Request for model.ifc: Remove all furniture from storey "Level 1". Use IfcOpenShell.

First a look at what the model holds.

```python
import ifcopenshell
import ifcopenshell.util.element

model = ifcopenshell.open("model.ifc")
print(model.schema)
storey = next(s for s in model.by_type("IfcBuildingStorey") if s.Name == "Level 1")
furniture = [e for e in ifcopenshell.util.element.get_decomposition(storey) if e.is_a("IfcFurnishingElement")]
seen = {}
for e in furniture:
    element_type = ifcopenshell.util.element.get_type(e)
    name = element_type.Name if element_type not in (None, e) else None
    seen[name] = seen.get(name, 0) + 1
for name, count in sorted(seen.items(), key=str):
    print(count, "x", name)
```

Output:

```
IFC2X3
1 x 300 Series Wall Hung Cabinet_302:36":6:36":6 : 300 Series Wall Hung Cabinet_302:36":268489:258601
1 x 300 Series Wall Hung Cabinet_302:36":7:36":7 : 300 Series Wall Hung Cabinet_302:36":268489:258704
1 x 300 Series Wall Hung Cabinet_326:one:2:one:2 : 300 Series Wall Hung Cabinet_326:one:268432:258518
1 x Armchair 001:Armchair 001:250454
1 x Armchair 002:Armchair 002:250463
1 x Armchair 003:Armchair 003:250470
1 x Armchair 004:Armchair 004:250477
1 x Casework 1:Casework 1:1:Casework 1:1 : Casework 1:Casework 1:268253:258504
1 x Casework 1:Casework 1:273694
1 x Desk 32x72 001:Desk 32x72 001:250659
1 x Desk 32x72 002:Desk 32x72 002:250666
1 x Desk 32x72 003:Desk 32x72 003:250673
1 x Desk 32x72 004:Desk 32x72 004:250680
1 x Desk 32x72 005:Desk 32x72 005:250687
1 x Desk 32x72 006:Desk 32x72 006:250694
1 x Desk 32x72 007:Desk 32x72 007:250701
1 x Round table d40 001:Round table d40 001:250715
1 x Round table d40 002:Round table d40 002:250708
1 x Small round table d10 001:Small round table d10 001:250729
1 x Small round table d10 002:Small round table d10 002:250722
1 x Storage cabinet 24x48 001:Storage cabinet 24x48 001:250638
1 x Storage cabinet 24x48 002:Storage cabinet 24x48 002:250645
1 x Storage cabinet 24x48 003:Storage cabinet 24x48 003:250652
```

```python
import ifcopenshell
import ifcopenshell.api.root
import ifcopenshell.util.element

model = ifcopenshell.open("model.ifc")

storey = next(s for s in model.by_type("IfcBuildingStorey") if s.Name == "Level 1")
furniture = [e for e in ifcopenshell.util.element.get_decomposition(storey) if e.is_a("IfcFurnishingElement")]

for e in furniture:
    ifcopenshell.api.root.remove_product(model, product=e)
print(len(furniture), "removed")

model.write("model-out.ifc")
```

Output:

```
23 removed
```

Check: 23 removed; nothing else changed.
